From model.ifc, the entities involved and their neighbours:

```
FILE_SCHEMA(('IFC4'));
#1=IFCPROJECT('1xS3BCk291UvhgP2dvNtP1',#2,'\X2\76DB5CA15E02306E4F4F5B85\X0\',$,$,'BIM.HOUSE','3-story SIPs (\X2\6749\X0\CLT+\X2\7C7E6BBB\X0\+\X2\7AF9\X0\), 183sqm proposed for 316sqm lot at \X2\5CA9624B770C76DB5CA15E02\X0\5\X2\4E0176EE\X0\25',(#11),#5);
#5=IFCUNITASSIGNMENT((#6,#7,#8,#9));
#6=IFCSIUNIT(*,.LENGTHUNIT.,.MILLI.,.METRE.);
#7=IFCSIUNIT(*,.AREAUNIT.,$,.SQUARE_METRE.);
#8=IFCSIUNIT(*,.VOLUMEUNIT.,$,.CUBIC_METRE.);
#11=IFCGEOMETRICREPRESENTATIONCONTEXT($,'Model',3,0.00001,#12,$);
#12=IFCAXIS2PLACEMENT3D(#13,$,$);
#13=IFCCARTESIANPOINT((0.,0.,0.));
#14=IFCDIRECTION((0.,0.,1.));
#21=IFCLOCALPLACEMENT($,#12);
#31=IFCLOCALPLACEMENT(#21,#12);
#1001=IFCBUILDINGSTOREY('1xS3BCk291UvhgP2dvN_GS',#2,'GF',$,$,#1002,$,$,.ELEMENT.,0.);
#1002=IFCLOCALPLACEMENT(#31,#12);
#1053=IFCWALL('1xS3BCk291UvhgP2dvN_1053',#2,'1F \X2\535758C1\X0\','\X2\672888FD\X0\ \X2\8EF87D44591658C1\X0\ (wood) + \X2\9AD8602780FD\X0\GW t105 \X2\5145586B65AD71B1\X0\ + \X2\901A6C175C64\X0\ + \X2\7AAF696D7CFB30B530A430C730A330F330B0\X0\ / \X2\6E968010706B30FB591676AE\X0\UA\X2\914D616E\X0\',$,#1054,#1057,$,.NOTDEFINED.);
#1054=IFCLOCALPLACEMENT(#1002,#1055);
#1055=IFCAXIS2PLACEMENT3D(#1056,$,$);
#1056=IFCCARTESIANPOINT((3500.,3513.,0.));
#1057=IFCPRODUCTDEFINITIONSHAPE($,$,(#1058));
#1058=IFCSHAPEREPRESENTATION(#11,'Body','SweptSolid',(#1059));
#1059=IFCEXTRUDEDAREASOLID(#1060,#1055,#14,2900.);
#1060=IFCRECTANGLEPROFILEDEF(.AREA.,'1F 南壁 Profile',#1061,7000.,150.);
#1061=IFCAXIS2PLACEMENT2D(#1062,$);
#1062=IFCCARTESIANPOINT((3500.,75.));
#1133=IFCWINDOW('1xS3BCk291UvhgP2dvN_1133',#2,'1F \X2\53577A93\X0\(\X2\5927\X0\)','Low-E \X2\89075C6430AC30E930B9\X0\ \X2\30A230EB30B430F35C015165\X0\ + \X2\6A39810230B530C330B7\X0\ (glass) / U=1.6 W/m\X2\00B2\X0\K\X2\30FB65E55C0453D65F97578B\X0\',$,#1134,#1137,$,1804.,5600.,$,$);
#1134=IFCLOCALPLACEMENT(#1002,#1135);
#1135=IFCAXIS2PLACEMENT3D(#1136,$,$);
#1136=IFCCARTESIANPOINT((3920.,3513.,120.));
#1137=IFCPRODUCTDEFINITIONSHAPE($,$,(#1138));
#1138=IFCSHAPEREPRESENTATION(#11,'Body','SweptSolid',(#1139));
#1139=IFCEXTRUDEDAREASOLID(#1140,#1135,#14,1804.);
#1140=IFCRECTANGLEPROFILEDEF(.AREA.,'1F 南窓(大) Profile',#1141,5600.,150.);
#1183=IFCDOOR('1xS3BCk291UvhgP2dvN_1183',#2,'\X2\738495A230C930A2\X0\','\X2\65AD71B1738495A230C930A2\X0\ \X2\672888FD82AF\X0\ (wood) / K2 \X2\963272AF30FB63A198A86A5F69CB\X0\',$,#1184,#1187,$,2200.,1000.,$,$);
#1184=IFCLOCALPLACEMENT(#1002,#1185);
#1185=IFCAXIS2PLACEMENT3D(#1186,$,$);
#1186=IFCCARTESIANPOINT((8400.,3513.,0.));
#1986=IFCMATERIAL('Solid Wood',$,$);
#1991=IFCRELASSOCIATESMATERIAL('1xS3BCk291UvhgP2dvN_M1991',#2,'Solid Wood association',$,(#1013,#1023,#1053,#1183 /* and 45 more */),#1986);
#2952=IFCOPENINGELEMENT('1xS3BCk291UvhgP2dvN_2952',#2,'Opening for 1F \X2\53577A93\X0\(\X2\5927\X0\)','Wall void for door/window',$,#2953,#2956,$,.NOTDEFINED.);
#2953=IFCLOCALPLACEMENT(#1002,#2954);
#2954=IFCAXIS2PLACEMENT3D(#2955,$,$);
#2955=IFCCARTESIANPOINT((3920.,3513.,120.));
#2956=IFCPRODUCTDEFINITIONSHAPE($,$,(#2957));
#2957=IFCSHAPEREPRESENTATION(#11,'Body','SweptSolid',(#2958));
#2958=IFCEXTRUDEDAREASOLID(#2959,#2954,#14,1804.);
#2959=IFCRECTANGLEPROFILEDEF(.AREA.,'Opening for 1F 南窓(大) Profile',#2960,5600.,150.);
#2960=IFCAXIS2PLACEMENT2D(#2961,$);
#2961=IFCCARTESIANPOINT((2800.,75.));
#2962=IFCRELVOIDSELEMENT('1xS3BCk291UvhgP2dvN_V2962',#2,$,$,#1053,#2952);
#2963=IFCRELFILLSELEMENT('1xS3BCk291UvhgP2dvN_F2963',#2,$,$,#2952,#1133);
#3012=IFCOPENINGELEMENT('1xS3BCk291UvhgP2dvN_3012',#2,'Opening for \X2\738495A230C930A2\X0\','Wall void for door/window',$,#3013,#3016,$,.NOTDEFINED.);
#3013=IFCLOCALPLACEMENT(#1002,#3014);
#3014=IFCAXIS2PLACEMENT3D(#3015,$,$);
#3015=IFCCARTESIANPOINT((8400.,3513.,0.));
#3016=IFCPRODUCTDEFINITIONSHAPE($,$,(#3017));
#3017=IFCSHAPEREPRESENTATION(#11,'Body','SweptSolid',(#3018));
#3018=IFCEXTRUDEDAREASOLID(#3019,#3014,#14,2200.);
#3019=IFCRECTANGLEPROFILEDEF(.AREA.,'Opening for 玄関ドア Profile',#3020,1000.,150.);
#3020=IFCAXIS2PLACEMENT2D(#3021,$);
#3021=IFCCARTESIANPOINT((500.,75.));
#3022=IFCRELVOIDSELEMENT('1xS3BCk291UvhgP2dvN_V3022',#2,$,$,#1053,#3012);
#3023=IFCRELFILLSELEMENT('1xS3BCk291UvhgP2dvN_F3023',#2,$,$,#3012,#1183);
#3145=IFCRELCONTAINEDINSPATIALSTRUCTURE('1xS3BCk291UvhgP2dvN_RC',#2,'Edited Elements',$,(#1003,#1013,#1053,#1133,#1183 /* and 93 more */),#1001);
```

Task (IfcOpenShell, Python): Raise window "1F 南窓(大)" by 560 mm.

```python
import numpy as np
import ifcopenshell
import ifcopenshell.api.geometry
import ifcopenshell.util.placement
import ifcopenshell.util.unit

model = ifcopenshell.open("model.ifc")
unit_scale = ifcopenshell.util.unit.calculate_unit_scale(model)

window = model.by_guid("1xS3BCk291UvhgP2dvN_1133")
opening = window.FillsVoids[0].RelatingOpeningElement
dz = 560.0

shift = np.array([0.0, 0.0, dz])
# The window is not placed relative to its opening, so move both.
for product in (opening, window):
    matrix = ifcopenshell.util.placement.get_local_placement(product.ObjectPlacement)
    matrix[:3, 3] += shift
    ifcopenshell.api.geometry.edit_object_placement(model, product=product, matrix=matrix, is_si=False)

print(f"moved by {dz * unit_scale:+.3f} m")

model.write("model_edited.ifc")
```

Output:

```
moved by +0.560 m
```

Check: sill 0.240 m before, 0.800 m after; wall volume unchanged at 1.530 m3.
